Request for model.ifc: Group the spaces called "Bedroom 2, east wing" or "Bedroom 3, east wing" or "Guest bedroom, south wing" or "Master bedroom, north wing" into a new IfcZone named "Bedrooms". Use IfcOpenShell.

First a look at what the model holds.

```python
import ifcopenshell

model = ifcopenshell.open("model.ifc")
print(model.schema)
seen = {}
for space in model.by_type("IfcSpace"):
    seen[space.LongName] = seen.get(space.LongName, 0) + 1
for name, count in sorted(seen.items(), key=str):
    print(count, "x", name)
print("zones:", [z.Name for z in model.by_type("IfcZone")][:20])
```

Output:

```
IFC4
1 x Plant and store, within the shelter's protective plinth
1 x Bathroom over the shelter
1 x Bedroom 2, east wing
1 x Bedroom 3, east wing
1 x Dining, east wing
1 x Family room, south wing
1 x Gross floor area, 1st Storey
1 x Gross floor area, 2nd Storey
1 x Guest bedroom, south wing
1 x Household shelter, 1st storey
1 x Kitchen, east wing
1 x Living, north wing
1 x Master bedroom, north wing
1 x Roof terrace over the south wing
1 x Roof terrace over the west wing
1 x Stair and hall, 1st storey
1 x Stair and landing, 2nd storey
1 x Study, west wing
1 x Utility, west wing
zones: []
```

```python
import ifcopenshell
import ifcopenshell.api.group
import ifcopenshell.api.root

model = ifcopenshell.open("model.ifc")

names = {"Bedroom 2, east wing", "Bedroom 3, east wing", "Guest bedroom, south wing", "Master bedroom, north wing"}
spaces = [s for s in model.by_type("IfcSpace") if s.LongName in names]

zone = ifcopenshell.api.root.create_entity(model, ifc_class="IfcZone", name="Bedrooms")
ifcopenshell.api.group.assign_group(model, products=spaces, group=zone)
print(len(spaces), "spaces in", zone.Name)

model.write("model_edited.ifc")
```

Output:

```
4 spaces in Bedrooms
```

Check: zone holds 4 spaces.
